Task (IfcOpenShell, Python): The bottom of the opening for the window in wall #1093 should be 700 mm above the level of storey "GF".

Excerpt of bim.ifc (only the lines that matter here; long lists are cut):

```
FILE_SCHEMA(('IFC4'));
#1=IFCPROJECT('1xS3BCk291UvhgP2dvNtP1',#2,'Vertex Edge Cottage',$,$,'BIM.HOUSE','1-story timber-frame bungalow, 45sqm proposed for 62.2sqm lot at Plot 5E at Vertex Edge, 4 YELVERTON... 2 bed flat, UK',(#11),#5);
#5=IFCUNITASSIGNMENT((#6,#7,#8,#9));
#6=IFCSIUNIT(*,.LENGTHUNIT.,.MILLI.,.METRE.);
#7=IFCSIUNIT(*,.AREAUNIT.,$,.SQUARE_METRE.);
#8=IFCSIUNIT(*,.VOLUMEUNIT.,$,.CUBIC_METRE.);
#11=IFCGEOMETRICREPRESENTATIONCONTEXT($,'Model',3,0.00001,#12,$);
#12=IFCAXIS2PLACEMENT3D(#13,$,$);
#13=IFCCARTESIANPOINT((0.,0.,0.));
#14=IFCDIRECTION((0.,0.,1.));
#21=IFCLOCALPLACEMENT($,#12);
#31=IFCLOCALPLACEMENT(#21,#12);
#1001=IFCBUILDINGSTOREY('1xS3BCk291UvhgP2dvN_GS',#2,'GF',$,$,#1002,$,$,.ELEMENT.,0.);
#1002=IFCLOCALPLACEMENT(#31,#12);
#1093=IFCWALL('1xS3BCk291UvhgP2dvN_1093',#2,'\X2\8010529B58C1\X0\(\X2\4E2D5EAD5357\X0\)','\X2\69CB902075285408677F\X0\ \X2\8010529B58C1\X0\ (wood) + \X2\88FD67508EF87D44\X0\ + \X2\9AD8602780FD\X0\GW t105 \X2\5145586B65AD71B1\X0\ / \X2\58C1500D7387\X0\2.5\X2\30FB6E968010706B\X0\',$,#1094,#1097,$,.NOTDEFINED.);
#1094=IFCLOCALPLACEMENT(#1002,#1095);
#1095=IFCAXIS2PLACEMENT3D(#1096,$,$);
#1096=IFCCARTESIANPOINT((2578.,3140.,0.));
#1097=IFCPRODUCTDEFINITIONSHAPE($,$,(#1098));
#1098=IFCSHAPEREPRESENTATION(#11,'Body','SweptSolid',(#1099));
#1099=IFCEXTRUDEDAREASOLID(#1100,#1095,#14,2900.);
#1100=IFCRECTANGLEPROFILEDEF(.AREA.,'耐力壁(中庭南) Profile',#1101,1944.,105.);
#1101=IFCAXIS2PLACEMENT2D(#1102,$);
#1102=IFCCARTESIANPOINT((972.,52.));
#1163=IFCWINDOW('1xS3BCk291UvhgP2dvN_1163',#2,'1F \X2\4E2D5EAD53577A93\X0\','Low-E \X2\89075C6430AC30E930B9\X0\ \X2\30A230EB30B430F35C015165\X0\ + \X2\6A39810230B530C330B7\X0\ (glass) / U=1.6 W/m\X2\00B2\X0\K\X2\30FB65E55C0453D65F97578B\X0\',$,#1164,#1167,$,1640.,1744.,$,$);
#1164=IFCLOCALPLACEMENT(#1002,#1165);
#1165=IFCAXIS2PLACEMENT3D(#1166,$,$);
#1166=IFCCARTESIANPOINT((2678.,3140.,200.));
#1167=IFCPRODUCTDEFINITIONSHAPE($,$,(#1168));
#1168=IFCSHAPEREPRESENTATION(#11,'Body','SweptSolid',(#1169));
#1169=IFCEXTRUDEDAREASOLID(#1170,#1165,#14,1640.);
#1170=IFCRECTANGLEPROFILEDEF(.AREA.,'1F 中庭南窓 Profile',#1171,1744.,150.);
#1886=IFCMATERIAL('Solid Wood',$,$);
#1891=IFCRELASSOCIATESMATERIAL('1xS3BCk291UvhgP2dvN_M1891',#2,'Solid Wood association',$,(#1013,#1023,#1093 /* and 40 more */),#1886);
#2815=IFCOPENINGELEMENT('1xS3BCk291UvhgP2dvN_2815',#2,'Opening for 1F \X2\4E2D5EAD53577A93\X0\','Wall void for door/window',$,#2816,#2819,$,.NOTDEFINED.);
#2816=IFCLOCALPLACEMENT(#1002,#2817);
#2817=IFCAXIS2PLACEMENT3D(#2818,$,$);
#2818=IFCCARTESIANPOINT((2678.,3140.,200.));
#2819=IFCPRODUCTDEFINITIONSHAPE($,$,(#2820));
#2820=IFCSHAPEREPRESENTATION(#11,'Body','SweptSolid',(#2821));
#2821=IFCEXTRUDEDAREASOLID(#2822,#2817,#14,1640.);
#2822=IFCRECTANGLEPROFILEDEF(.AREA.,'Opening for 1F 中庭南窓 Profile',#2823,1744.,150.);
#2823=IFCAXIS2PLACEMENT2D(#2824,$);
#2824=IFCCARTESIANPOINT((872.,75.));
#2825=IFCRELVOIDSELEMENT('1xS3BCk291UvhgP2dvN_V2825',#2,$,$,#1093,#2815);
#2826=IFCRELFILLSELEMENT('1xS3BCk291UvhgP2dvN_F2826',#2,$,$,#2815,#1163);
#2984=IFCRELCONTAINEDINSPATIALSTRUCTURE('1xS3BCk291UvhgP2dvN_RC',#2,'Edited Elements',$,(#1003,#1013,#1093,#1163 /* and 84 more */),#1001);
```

```python
import numpy as np
import ifcopenshell
import ifcopenshell.api.geometry
import ifcopenshell.geom
import ifcopenshell.util.element
import ifcopenshell.util.placement
import ifcopenshell.util.shape
import ifcopenshell.util.unit

model = ifcopenshell.open("bim.ifc")
unit_scale = ifcopenshell.util.unit.calculate_unit_scale(model)

window = model.by_guid("1xS3BCk291UvhgP2dvN_1163")
opening = window.FillsVoids[0].RelatingOpeningElement
storey = ifcopenshell.util.element.get_container(window, ifc_class="IfcBuildingStorey")
level = ifcopenshell.util.placement.get_local_placement(storey.ObjectPlacement)[2, 3]

# The opening's origin need not be at the sill, so measure its lowest point.
shape = ifcopenshell.geom.create_shape(ifcopenshell.geom.settings(), opening)
bottom = ifcopenshell.util.shape.get_shape_bottom_elevation(shape, shape.geometry) / unit_scale
dz = level + 700.0 - bottom

shift = np.array([0.0, 0.0, dz])
# The window is not placed relative to its opening, so move both.
for product in (opening, window):
    matrix = ifcopenshell.util.placement.get_local_placement(product.ObjectPlacement)
    matrix[:3, 3] += shift
    ifcopenshell.api.geometry.edit_object_placement(model, product=product, matrix=matrix, is_si=False)

print(f"moved by {dz * unit_scale:+.3f} m")

model.write("bim_edited.ifc")
```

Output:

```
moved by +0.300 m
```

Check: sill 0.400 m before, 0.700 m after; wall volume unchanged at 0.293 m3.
